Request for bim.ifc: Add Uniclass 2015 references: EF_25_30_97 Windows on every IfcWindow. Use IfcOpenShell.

First a look at what the model holds.

```python
import ifcopenshell

model = ifcopenshell.open("bim.ifc")
print(model.schema)
print("classifications:", [c.Name for c in model.by_type("IfcClassification")])
for ifc_class in ("IfcDoor", "IfcRoof", "IfcStair", "IfcWall", "IfcWindow"):
    print(ifc_class, len(model.by_type(ifc_class)))
```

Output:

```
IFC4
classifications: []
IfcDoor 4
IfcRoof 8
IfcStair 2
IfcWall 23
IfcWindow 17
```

```python
import ifcopenshell
import ifcopenshell.api.classification

model = ifcopenshell.open("bim.ifc")

system = ifcopenshell.api.classification.add_classification(model, classification="Uniclass 2015")

codes = {
    "IfcWindow": ("EF_25_30_97", "Windows"),
}
for ifc_class, (code, name) in codes.items():
    products = model.by_type(ifc_class)
    ifcopenshell.api.classification.add_reference(
        model, products=products, classification=system, identification=code, name=name
    )
    print(code, len(products))

model.write("bim_v2.ifc")
```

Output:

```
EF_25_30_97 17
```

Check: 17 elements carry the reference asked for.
